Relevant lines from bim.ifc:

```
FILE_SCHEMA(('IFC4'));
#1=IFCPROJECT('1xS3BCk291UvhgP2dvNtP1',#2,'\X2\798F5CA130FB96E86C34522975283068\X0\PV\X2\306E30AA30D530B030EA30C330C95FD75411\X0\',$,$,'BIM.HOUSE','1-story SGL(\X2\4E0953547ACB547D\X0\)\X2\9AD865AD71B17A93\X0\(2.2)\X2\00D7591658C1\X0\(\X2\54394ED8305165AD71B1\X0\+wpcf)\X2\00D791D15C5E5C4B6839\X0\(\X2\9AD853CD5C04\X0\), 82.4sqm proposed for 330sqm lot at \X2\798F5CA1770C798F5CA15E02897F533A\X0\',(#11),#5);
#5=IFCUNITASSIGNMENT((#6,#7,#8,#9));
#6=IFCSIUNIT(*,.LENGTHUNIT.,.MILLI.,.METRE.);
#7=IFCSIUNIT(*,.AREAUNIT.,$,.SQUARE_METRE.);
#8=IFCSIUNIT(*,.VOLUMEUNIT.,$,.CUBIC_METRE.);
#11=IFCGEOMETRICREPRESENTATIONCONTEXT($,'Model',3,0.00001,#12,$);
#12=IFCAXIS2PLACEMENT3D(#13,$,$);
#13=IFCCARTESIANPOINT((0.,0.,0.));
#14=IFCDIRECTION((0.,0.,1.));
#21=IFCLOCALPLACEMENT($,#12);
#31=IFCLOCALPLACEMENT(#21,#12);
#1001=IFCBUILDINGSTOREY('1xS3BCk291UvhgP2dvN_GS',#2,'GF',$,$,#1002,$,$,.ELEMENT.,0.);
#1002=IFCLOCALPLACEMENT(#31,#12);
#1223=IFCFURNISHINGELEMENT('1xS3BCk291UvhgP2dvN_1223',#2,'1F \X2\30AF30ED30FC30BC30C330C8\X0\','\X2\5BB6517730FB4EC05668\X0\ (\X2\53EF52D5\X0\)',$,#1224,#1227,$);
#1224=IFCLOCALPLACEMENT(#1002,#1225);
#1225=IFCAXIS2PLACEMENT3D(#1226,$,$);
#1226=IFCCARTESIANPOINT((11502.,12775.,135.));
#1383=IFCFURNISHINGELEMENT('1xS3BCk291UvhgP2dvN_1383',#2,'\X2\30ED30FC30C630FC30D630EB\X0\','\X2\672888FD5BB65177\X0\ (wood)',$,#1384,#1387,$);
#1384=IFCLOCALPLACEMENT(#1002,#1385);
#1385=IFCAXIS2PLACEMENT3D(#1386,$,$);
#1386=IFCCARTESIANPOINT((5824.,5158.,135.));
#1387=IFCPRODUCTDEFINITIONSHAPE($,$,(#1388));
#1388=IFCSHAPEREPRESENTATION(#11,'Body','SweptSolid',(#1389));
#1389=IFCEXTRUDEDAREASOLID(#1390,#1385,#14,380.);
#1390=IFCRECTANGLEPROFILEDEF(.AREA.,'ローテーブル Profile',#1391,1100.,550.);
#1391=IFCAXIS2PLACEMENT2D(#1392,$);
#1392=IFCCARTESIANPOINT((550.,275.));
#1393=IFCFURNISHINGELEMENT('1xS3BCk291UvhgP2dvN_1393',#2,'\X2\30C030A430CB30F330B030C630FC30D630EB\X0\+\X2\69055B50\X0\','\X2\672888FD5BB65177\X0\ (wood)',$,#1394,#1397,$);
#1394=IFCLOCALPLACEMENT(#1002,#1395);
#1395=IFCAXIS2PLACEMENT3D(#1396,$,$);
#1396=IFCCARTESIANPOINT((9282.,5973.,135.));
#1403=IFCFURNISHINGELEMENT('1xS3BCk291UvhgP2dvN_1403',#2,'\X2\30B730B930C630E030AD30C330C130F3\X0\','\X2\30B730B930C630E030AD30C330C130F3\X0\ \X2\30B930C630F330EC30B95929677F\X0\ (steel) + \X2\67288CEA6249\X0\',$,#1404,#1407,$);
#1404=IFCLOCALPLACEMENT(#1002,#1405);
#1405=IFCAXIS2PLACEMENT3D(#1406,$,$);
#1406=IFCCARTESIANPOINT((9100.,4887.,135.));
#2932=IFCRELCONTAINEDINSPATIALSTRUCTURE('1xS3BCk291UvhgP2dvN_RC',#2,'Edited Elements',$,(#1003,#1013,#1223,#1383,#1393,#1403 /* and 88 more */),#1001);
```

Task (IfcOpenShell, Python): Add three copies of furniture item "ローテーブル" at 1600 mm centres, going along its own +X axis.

```python
import ifcopenshell
import ifcopenshell.api.geometry
import ifcopenshell.api.root
import ifcopenshell.util.element
import ifcopenshell.util.placement
import ifcopenshell.util.unit

model = ifcopenshell.open("bim.ifc")
unit_scale = ifcopenshell.util.unit.calculate_unit_scale(model)


def reuse_history(source, copy):
    """copy_class also copies each property set's owner history, people and application; keep the originals."""
    for rel in copy.IsDefinedBy:
        if rel.is_a("IfcRelDefinesByProperties") and (history := rel.RelatingPropertyDefinition.OwnerHistory):
            rel.RelatingPropertyDefinition.OwnerHistory = source.OwnerHistory
            ifcopenshell.util.element.remove_deep2(model, history)


source = model.by_id(1383)
base = ifcopenshell.util.placement.get_local_placement(source.ObjectPlacement)
step = base[:3, 0] * 1.6 / unit_scale

for i in range(1, 4):
    copy = ifcopenshell.api.root.copy_class(model, product=source)
    copy.Representation = ifcopenshell.util.element.copy_deep(
        model, source.Representation, exclude=["IfcGeometricRepresentationContext", "IfcRepresentationMap"]
    )
    reuse_history(source, copy)
    matrix = base.copy()
    matrix[:3, 3] += i * step
    print("added at", matrix[:3, 3].round(3) + 0.0)
    ifcopenshell.api.geometry.edit_object_placement(model, product=copy, matrix=matrix, is_si=False)

model.write("bim-out.ifc")
```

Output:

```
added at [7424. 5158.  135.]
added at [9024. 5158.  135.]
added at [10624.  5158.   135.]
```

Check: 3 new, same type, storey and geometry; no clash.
